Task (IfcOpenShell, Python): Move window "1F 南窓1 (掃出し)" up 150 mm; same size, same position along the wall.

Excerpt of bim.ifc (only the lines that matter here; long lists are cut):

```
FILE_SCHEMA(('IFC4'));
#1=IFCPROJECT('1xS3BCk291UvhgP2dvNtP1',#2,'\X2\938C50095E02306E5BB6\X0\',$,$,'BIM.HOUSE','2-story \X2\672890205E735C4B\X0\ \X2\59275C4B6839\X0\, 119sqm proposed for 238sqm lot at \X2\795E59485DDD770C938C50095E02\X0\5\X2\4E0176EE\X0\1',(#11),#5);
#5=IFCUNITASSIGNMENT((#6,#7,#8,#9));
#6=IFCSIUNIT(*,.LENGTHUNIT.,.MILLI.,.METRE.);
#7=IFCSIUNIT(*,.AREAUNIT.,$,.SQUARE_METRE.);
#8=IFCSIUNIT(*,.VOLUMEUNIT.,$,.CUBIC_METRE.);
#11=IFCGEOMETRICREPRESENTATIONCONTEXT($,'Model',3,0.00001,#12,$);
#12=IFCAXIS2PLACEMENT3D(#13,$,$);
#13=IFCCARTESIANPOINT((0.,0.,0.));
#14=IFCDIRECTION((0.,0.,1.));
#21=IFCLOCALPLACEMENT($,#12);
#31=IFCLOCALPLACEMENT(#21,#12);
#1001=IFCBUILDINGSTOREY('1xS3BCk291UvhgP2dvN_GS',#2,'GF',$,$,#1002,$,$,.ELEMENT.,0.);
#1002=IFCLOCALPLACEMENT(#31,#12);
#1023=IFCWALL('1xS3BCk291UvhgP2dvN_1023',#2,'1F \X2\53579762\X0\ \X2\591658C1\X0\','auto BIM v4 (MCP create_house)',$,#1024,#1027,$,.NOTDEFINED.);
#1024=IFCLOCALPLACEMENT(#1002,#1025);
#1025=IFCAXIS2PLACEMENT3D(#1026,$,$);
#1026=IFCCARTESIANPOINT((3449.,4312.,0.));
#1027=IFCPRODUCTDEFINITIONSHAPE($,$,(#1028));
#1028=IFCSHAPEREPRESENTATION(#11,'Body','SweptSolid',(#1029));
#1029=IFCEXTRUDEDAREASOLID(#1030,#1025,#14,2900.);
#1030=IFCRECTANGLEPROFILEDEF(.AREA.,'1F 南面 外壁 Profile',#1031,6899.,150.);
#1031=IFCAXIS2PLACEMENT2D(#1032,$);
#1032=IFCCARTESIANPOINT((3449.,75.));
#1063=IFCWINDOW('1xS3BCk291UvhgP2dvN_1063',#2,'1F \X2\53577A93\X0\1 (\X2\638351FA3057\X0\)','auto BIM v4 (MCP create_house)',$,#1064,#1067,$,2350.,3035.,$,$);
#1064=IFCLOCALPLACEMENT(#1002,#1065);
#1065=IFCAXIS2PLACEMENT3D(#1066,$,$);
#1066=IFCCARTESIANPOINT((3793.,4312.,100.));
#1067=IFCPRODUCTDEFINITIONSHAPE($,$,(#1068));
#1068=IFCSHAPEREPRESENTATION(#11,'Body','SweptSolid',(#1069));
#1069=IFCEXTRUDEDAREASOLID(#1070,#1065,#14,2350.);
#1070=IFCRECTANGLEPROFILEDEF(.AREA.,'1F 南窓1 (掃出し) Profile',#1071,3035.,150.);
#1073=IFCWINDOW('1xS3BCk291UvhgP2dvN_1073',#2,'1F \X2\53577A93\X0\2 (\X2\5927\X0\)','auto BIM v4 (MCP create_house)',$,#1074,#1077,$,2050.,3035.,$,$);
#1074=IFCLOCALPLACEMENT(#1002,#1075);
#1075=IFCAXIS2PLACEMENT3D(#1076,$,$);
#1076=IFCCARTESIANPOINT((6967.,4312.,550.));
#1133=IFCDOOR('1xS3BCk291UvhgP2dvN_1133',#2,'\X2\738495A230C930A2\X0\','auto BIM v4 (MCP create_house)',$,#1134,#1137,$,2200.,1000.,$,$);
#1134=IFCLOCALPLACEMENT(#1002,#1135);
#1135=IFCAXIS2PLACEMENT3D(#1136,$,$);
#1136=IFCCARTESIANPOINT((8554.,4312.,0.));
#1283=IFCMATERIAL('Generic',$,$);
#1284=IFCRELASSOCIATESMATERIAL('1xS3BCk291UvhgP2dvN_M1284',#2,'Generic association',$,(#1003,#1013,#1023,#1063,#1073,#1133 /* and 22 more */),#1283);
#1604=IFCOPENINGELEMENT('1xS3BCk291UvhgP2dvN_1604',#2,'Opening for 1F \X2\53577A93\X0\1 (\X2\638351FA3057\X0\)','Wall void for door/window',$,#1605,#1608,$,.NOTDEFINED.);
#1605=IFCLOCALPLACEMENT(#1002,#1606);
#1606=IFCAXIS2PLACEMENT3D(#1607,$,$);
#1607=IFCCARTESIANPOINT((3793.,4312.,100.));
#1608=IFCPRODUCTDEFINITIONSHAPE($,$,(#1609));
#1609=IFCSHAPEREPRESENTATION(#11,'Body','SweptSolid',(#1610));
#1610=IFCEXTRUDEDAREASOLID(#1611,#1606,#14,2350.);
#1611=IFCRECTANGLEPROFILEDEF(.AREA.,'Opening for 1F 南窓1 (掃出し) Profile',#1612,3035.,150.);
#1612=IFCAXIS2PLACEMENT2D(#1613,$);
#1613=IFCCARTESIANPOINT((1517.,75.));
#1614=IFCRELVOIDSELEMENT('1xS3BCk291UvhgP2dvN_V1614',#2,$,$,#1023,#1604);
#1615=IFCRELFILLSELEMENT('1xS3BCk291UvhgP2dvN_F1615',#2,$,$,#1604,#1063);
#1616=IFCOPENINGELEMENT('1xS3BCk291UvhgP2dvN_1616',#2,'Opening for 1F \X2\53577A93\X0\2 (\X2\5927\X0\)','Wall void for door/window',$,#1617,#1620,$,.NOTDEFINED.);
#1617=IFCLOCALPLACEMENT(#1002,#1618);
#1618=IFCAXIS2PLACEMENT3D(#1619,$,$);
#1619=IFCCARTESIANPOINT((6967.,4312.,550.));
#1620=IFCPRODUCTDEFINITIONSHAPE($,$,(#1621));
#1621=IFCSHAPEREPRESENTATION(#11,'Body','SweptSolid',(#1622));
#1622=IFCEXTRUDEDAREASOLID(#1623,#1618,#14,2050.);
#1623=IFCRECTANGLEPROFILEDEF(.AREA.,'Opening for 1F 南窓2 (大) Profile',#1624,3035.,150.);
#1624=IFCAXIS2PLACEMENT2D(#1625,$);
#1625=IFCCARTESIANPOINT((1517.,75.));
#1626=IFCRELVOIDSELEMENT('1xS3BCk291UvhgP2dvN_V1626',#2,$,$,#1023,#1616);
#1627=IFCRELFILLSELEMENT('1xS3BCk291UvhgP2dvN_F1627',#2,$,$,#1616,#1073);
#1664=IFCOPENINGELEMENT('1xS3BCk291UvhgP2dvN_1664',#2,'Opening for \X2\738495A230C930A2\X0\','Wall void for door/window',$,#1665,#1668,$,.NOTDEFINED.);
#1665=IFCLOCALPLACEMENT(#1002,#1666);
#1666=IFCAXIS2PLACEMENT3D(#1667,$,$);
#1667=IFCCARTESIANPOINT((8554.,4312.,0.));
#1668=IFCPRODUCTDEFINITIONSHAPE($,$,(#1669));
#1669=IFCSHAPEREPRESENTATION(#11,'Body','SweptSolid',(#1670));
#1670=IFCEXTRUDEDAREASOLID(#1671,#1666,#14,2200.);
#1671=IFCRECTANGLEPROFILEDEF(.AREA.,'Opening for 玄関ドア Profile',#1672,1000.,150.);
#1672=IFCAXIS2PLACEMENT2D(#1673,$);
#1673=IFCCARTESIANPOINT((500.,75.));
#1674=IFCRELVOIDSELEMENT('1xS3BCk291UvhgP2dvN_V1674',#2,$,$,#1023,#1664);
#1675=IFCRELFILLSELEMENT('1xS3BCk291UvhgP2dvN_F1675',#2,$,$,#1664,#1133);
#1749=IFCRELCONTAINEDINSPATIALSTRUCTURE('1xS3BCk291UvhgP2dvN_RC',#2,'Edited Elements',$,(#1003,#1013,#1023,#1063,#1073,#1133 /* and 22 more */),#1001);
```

```python
import numpy as np
import ifcopenshell
import ifcopenshell.api.geometry
import ifcopenshell.util.placement
import ifcopenshell.util.unit

model = ifcopenshell.open("bim.ifc")
unit_scale = ifcopenshell.util.unit.calculate_unit_scale(model)

window = model.by_guid("1xS3BCk291UvhgP2dvN_1063")
opening = window.FillsVoids[0].RelatingOpeningElement
dz = 150.0

shift = np.array([0.0, 0.0, dz])
# The window is not placed relative to its opening, so move both.
for product in (opening, window):
    matrix = ifcopenshell.util.placement.get_local_placement(product.ObjectPlacement)
    matrix[:3, 3] += shift
    ifcopenshell.api.geometry.edit_object_placement(model, product=product, matrix=matrix, is_si=False)

print(f"moved by {dz * unit_scale:+.3f} m")

model.write("bim_rev.ifc")
```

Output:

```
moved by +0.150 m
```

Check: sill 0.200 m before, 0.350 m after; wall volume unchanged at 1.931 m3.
